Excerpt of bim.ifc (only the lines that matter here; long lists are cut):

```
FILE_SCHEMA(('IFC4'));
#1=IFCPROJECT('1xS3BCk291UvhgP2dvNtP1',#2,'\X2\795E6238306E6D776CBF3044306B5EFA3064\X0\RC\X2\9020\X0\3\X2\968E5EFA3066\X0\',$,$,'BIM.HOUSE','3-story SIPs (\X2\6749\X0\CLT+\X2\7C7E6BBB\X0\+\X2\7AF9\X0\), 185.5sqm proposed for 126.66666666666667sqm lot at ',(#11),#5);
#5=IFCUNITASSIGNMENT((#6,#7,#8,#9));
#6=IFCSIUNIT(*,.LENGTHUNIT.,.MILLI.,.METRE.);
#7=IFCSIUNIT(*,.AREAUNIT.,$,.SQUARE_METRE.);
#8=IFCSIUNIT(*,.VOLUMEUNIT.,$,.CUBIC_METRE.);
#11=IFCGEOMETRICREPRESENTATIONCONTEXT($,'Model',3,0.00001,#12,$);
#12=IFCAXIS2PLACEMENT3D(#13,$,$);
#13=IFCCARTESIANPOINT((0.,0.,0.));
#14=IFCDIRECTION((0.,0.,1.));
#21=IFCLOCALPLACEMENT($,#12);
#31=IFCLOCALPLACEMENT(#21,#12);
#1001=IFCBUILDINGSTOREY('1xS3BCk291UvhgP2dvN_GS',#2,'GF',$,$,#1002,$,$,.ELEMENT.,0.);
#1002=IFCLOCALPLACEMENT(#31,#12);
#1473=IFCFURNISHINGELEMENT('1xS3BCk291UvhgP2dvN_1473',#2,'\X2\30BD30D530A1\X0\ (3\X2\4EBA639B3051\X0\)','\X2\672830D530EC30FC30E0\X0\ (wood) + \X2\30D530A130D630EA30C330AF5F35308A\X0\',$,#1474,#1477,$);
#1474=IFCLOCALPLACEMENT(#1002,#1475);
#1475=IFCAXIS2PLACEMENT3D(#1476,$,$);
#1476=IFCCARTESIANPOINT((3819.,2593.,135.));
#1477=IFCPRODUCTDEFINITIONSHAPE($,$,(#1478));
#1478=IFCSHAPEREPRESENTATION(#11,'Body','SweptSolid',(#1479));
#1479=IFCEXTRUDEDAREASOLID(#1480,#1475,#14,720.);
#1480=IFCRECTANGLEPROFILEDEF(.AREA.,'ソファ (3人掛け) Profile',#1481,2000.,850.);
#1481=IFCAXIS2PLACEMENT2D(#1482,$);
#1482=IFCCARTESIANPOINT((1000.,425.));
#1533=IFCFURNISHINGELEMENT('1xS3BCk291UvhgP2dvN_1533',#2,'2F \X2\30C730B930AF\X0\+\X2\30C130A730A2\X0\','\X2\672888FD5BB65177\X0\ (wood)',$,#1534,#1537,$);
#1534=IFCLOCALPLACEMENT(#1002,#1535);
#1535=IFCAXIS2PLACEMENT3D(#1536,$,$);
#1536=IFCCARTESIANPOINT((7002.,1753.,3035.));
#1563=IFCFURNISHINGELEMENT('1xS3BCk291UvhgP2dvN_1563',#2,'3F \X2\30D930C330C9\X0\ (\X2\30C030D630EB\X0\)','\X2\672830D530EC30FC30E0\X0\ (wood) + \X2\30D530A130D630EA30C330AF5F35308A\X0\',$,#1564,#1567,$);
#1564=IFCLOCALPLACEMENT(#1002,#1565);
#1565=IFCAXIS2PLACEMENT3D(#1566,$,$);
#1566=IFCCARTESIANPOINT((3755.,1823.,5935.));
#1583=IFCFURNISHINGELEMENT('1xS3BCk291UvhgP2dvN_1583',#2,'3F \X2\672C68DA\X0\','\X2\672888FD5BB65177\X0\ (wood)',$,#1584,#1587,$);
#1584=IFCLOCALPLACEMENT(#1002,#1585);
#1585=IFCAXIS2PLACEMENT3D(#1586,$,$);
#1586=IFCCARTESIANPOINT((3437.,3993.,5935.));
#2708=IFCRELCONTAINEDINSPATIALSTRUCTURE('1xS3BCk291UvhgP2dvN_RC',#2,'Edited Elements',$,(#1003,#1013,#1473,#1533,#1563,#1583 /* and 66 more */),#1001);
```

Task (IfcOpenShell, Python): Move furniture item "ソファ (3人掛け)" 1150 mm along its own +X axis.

```python
import ifcopenshell
import ifcopenshell.api.geometry
import ifcopenshell.util.placement
import ifcopenshell.util.unit

model = ifcopenshell.open("bim.ifc")
unit_scale = ifcopenshell.util.unit.calculate_unit_scale(model)

item = model.by_guid("1xS3BCk291UvhgP2dvN_1473")
matrix = ifcopenshell.util.placement.get_local_placement(item.ObjectPlacement)
matrix[:3, 3] += matrix[:3, 0] * 1.15 / unit_scale
ifcopenshell.api.geometry.edit_object_placement(model, product=item, matrix=matrix, is_si=False)

print(ifcopenshell.util.placement.get_local_placement(item.ObjectPlacement).round(3) + 0.0)

model.write("bim_updated.ifc")
```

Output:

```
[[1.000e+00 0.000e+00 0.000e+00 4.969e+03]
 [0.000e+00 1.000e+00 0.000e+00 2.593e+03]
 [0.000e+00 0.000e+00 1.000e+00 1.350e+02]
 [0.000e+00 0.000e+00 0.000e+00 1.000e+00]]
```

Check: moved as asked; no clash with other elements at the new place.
